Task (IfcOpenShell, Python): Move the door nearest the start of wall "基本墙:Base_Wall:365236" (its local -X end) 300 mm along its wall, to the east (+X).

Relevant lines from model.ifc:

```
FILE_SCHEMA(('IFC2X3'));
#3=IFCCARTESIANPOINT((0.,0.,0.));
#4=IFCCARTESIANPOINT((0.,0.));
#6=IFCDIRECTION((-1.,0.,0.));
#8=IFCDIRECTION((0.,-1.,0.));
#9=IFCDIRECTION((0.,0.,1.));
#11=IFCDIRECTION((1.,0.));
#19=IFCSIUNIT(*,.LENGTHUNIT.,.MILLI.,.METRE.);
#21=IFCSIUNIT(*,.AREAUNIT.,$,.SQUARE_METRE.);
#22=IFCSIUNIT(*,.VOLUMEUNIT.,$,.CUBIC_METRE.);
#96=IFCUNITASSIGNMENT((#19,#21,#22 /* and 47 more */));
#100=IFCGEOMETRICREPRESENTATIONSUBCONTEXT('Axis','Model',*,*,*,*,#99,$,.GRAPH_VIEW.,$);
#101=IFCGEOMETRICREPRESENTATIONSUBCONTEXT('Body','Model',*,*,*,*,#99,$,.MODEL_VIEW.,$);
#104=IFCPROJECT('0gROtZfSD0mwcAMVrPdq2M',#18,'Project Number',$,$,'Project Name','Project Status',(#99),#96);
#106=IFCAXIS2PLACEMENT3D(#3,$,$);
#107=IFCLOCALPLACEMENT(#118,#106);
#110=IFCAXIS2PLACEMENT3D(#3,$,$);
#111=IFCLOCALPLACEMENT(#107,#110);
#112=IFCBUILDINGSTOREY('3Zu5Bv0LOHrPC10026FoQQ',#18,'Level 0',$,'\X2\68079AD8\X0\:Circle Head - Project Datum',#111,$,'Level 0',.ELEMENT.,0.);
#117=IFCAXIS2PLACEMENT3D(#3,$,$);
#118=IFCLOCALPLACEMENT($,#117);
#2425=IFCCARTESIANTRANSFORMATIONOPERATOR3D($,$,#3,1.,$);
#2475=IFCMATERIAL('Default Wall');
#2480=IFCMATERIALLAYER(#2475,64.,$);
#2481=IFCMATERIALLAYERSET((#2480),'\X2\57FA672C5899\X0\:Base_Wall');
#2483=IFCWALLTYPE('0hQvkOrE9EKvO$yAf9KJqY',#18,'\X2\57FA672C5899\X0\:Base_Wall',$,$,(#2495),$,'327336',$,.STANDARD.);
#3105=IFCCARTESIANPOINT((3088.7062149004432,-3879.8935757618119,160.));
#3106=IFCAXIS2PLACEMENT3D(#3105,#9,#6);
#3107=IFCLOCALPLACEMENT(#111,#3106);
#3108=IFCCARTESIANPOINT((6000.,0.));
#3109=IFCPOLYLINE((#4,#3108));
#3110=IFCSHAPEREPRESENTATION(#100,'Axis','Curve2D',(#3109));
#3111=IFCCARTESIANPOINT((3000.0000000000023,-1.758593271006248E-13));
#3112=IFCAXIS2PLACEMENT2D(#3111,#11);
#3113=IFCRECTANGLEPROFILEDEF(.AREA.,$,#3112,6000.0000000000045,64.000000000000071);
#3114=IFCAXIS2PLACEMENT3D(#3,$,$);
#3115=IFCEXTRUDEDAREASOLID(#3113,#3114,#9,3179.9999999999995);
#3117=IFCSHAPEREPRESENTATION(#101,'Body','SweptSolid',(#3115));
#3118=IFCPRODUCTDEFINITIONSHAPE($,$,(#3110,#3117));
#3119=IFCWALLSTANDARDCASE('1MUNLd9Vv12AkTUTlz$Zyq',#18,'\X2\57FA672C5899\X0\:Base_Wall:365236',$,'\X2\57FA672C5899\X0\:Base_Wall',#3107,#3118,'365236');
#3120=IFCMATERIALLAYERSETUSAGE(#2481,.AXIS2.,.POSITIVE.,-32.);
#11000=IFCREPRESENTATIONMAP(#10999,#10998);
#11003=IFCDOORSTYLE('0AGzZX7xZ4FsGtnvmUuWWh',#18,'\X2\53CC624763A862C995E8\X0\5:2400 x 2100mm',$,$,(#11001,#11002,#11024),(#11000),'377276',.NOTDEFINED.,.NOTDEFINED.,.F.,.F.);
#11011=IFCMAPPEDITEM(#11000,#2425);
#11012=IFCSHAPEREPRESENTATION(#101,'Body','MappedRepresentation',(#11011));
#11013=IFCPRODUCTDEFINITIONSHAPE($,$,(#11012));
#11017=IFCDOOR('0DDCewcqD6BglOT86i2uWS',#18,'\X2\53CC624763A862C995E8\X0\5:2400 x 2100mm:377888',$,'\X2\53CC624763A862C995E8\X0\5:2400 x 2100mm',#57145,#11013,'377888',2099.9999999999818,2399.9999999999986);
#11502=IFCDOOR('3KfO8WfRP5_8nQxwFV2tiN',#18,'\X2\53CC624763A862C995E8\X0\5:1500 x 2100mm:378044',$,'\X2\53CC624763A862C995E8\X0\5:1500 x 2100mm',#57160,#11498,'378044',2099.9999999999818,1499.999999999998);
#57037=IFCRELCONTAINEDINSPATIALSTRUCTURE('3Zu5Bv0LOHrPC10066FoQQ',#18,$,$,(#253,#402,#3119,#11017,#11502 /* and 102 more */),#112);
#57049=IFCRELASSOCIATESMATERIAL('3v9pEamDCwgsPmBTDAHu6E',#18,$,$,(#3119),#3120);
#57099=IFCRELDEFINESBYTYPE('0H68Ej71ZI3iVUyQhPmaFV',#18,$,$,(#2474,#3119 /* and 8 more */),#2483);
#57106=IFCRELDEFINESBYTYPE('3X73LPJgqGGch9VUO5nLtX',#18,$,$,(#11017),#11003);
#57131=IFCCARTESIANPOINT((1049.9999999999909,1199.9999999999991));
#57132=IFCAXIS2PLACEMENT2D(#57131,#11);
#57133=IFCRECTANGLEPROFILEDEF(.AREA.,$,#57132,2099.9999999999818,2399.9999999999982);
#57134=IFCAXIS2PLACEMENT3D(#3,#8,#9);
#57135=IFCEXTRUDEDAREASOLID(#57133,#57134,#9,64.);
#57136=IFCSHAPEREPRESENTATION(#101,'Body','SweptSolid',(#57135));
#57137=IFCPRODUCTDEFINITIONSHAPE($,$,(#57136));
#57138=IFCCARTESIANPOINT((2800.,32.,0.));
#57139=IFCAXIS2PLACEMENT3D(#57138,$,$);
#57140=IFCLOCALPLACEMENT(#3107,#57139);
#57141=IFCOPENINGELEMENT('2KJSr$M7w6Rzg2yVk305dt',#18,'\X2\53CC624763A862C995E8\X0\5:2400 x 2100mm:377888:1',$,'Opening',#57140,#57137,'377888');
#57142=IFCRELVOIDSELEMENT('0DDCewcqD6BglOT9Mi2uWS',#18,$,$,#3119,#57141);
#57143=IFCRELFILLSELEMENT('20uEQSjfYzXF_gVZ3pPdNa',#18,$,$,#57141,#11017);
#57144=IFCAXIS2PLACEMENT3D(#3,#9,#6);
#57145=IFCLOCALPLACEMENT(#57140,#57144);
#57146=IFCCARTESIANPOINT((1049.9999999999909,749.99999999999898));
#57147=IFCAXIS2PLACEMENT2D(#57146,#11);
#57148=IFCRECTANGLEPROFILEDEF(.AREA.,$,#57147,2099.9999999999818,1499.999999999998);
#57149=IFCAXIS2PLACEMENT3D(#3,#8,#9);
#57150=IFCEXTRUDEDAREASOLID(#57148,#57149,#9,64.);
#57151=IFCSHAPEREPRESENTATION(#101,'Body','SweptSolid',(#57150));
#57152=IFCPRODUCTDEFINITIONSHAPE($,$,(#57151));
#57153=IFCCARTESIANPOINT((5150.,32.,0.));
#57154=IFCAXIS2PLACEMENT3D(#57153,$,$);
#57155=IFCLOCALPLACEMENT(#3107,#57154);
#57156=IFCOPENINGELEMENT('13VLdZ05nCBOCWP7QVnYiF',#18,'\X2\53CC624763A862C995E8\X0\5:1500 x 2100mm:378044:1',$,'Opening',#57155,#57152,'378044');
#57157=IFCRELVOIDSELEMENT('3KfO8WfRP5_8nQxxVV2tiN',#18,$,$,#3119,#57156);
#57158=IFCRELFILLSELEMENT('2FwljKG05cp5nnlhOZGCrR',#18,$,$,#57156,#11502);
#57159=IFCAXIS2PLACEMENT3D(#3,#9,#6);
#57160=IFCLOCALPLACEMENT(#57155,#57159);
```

```python
import ifcopenshell
import ifcopenshell.api.geometry
import ifcopenshell.util.placement
import ifcopenshell.util.unit

model = ifcopenshell.open("model.ifc")
unit_scale = ifcopenshell.util.unit.calculate_unit_scale(model)

door = model.by_guid("0DDCewcqD6BglOT86i2uWS")
opening = door.FillsVoids[0].RelatingOpeningElement
wall = opening.VoidsElements[0].RelatingBuildingElement

wall_matrix = ifcopenshell.util.placement.get_local_placement(wall.ObjectPlacement)
shift = wall_matrix[:3, 0] * -0.3 / unit_scale
before = ifcopenshell.util.placement.get_local_placement(door.ObjectPlacement)[:3, 3].copy()

# The door is placed relative to its opening, so it follows when the opening moves.
matrix = ifcopenshell.util.placement.get_local_placement(opening.ObjectPlacement)
matrix[:3, 3] += shift
ifcopenshell.api.geometry.edit_object_placement(
    model, product=opening, matrix=matrix, is_si=False, should_transform_children=True
)

after = ifcopenshell.util.placement.get_local_placement(door.ObjectPlacement)[:3, 3]
print("door moved by", (after - before).round(3) + 0.0)

model.write("model_edited.ifc")
```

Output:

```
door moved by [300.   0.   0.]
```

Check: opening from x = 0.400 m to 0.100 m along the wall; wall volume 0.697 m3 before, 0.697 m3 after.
